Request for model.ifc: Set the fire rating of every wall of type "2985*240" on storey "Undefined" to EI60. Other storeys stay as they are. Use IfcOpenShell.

First a look at what the model holds.

```python
import ifcopenshell
import ifcopenshell.util.element

model = ifcopenshell.open("model.ifc")
print(model.schema)
storey = next(s for s in model.by_type("IfcBuildingStorey") if s.Name == "Undefined")
walls = [e for e in ifcopenshell.util.element.get_decomposition(storey) if e.is_a("IfcWall")]
seen = {}
for e in walls:
    element_type = ifcopenshell.util.element.get_type(e)
    key = (element_type.Name if element_type != e and element_type else None, ifcopenshell.util.element.get_pset(e, "Pset_WallCommon", "FireRating"))
    seen[key] = seen.get(key, 0) + 1
for (name, value), count in sorted(seen.items(), key=str):
    print(count, "x", name, "|", value)
```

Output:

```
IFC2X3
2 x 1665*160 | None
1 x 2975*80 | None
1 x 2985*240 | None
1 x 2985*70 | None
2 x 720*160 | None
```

```python
import ifcopenshell
import ifcopenshell.api.pset
import ifcopenshell.util.element

model = ifcopenshell.open("model.ifc")

storey = next(s for s in model.by_type("IfcBuildingStorey") if s.Name == "Undefined")
walls = [e for e in ifcopenshell.util.element.get_decomposition(storey) if e.is_a("IfcWall")]

count = 0
for e in walls:
    element_type = ifcopenshell.util.element.get_type(e)
    if element_type in (None, e) or element_type.Name != "2985*240":
        continue
    # add_pset returns the element's existing set when there is one.
    pset = ifcopenshell.api.pset.add_pset(model, product=e, name="Pset_WallCommon")
    ifcopenshell.api.pset.edit_pset(model, pset=pset, properties={"FireRating": "EI60"})
    count += 1

print(count, "walls updated")

model.write("model_edited.ifc")
```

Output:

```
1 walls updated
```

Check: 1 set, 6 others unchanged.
